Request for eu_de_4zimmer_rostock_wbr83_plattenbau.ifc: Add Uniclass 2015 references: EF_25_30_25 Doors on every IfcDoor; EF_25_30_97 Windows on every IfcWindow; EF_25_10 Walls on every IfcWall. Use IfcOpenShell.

First a look at what the model holds.

```python
import ifcopenshell

model = ifcopenshell.open("eu_de_4zimmer_rostock_wbr83_plattenbau.ifc")
print(model.schema)
print("classifications:", [c.Name for c in model.by_type("IfcClassification")])
for ifc_class in ("IfcDoor", "IfcRoof", "IfcStair", "IfcWall", "IfcWindow"):
    print(ifc_class, len(model.by_type(ifc_class)))
```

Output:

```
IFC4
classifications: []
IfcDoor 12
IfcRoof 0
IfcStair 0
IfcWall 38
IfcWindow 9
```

```python
import ifcopenshell
import ifcopenshell.api.classification

model = ifcopenshell.open("eu_de_4zimmer_rostock_wbr83_plattenbau.ifc")

system = ifcopenshell.api.classification.add_classification(model, classification="Uniclass 2015")

codes = {
    "IfcDoor": ("EF_25_30_25", "Doors"),
    "IfcWindow": ("EF_25_30_97", "Windows"),
    "IfcWall": ("EF_25_10", "Walls"),
}
for ifc_class, (code, name) in codes.items():
    products = model.by_type(ifc_class)
    ifcopenshell.api.classification.add_reference(
        model, products=products, classification=system, identification=code, name=name
    )
    print(code, len(products))

model.write("eu_de_4zimmer_rostock_wbr83_plattenbau_edited.ifc")
```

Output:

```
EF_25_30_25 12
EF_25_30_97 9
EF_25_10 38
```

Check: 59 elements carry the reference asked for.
